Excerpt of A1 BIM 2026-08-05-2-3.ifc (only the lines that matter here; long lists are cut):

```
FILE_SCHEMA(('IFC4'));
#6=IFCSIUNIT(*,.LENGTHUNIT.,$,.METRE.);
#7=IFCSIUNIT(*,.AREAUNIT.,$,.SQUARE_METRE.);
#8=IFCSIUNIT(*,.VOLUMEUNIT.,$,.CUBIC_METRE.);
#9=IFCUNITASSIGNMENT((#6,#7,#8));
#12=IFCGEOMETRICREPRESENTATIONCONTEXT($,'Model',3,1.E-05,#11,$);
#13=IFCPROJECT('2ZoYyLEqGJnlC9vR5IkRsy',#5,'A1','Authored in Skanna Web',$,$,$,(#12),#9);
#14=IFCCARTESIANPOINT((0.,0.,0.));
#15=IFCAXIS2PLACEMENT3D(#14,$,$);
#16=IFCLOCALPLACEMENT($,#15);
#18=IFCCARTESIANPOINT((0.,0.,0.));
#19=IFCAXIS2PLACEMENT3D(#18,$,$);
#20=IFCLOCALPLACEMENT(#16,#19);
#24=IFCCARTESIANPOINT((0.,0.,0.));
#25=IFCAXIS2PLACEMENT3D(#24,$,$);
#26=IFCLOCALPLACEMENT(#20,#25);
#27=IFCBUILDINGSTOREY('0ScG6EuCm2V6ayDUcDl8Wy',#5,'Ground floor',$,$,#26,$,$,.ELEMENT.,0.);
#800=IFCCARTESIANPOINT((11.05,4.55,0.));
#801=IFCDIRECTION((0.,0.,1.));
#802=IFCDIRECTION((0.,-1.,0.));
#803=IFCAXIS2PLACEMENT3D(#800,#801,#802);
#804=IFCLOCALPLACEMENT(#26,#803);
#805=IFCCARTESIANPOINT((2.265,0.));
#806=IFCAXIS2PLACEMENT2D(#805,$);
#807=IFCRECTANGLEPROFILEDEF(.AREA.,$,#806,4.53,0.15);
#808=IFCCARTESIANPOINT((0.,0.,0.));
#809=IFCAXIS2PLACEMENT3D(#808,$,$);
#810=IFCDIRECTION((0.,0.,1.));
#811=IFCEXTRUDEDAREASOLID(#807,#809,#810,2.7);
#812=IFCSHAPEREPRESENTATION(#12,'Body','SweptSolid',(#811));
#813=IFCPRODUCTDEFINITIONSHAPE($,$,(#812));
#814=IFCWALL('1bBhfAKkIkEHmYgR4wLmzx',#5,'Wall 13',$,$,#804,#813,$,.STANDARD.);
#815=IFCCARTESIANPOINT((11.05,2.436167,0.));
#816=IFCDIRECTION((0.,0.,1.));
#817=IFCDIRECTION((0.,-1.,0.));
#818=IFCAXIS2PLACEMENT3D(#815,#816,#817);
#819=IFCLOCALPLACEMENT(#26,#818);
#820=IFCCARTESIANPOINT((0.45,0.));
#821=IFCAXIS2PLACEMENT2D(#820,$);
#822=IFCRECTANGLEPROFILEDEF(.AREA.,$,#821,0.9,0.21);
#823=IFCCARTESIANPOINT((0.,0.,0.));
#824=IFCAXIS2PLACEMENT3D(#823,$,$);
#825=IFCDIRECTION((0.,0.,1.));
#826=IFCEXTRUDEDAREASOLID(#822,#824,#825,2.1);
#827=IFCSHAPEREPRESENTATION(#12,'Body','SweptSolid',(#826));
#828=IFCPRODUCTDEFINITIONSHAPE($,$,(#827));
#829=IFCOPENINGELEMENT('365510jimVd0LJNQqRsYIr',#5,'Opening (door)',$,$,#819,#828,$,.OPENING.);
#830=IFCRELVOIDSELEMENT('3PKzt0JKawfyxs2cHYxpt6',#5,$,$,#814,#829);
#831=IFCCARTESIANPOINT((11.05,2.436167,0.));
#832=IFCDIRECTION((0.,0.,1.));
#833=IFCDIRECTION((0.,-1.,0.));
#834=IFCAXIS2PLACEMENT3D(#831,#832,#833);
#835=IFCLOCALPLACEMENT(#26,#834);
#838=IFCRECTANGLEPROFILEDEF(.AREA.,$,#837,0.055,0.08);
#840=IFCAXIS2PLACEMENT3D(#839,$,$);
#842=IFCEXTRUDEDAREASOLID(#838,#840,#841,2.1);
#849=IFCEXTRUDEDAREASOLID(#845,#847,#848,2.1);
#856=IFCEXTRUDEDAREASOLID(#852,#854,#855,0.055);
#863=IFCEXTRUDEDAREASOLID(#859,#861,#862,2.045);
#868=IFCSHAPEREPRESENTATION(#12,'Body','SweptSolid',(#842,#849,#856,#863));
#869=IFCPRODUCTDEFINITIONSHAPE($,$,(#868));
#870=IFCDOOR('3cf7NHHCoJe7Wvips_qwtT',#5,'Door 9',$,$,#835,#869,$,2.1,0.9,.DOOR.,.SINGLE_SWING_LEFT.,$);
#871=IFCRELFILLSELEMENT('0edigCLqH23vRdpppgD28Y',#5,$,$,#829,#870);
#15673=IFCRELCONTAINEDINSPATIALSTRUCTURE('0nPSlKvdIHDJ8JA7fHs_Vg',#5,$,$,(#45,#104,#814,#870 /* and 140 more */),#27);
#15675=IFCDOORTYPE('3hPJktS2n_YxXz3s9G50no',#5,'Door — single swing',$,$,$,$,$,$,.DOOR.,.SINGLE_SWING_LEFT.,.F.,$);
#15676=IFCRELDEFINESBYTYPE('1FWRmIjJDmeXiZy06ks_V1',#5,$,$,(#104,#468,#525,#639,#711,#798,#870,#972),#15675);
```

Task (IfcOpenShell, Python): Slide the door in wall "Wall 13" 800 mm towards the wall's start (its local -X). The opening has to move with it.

```python
import ifcopenshell
import ifcopenshell.api.geometry
import ifcopenshell.util.placement

model = ifcopenshell.open("A1 BIM 2026-08-05-2-3.ifc")

door = model.by_guid("3cf7NHHCoJe7Wvips_qwtT")
opening = door.FillsVoids[0].RelatingOpeningElement
wall = opening.VoidsElements[0].RelatingBuildingElement

wall_matrix = ifcopenshell.util.placement.get_local_placement(wall.ObjectPlacement)
shift = wall_matrix[:3, 0] * -0.8
before = ifcopenshell.util.placement.get_local_placement(door.ObjectPlacement)[:3, 3].copy()

# The door is not placed relative to its opening, so move both.
for product in (opening, door):
    matrix = ifcopenshell.util.placement.get_local_placement(product.ObjectPlacement)
    matrix[:3, 3] += shift
    ifcopenshell.api.geometry.edit_object_placement(model, product=product, matrix=matrix, is_si=False)

after = ifcopenshell.util.placement.get_local_placement(door.ObjectPlacement)[:3, 3]
print("door moved by", (after - before).round(3) + 0.0)

model.write("A1 BIM 2026-08-05-2-3_rev.ifc")
```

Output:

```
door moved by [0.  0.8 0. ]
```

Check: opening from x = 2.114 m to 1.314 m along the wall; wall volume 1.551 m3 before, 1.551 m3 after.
